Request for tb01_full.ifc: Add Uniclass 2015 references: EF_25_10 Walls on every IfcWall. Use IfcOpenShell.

First a look at what the model holds.

```python
import ifcopenshell

model = ifcopenshell.open("tb01_full.ifc")
print(model.schema)
print("classifications:", [c.Name for c in model.by_type("IfcClassification")])
for ifc_class in ("IfcDoor", "IfcRoof", "IfcStair", "IfcWall", "IfcWindow"):
    print(ifc_class, len(model.by_type(ifc_class)))
```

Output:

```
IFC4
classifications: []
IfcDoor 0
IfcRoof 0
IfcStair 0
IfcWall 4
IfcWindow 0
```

```python
import ifcopenshell
import ifcopenshell.api.classification

model = ifcopenshell.open("tb01_full.ifc")

system = ifcopenshell.api.classification.add_classification(model, classification="Uniclass 2015")

codes = {
    "IfcWall": ("EF_25_10", "Walls"),
}
for ifc_class, (code, name) in codes.items():
    products = model.by_type(ifc_class)
    ifcopenshell.api.classification.add_reference(
        model, products=products, classification=system, identification=code, name=name
    )
    print(code, len(products))

model.write("tb01_full-out.ifc")
```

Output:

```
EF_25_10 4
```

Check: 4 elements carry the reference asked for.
